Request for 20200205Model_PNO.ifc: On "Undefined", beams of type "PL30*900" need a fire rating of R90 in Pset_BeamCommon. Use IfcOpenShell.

First a look at what the model holds.

```python
import ifcopenshell
import ifcopenshell.util.element

model = ifcopenshell.open("20200205Model_PNO.ifc")
print(model.schema)
storey = next(s for s in model.by_type("IfcBuildingStorey") if s.Name == "Undefined")
beams = [e for e in ifcopenshell.util.element.get_decomposition(storey) if e.is_a("IfcBeam")]
seen = {}
for e in beams:
    element_type = ifcopenshell.util.element.get_type(e)
    key = (element_type.Name if element_type != e and element_type else None, ifcopenshell.util.element.get_pset(e, "Pset_BeamCommon", "FireRating"))
    seen[key] = seen.get(key, 0) + 1
for (name, value), count in sorted(seen.items(), key=str):
    print(count, "x", name, "|", value)
```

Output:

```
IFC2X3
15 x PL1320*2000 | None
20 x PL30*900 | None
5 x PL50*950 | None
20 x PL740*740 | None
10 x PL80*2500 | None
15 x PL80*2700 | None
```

```python
import ifcopenshell
import ifcopenshell.api.pset
import ifcopenshell.util.element

model = ifcopenshell.open("20200205Model_PNO.ifc")

storey = next(s for s in model.by_type("IfcBuildingStorey") if s.Name == "Undefined")
beams = [e for e in ifcopenshell.util.element.get_decomposition(storey) if e.is_a("IfcBeam")]

count = 0
for e in beams:
    element_type = ifcopenshell.util.element.get_type(e)
    if element_type in (None, e) or element_type.Name != "PL30*900":
        continue
    found = ifcopenshell.util.element.get_pset(e, "Pset_BeamCommon", should_inherit=False)
    if found:
        pset = model.by_id(found["id"])
        if len(ifcopenshell.util.element.get_elements_by_pset(pset)) > 1:
            pset = ifcopenshell.api.pset.unshare_pset(model, products=[e], pset=pset)[0]
    else:
        pset = ifcopenshell.api.pset.add_pset(model, product=e, name="Pset_BeamCommon")
    ifcopenshell.api.pset.edit_pset(model, pset=pset, properties={"FireRating": "R90"})
    count += 1

print(count, "beams updated")

model.write("20200205Model_PNO_v2.ifc")
```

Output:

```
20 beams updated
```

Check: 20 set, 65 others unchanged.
